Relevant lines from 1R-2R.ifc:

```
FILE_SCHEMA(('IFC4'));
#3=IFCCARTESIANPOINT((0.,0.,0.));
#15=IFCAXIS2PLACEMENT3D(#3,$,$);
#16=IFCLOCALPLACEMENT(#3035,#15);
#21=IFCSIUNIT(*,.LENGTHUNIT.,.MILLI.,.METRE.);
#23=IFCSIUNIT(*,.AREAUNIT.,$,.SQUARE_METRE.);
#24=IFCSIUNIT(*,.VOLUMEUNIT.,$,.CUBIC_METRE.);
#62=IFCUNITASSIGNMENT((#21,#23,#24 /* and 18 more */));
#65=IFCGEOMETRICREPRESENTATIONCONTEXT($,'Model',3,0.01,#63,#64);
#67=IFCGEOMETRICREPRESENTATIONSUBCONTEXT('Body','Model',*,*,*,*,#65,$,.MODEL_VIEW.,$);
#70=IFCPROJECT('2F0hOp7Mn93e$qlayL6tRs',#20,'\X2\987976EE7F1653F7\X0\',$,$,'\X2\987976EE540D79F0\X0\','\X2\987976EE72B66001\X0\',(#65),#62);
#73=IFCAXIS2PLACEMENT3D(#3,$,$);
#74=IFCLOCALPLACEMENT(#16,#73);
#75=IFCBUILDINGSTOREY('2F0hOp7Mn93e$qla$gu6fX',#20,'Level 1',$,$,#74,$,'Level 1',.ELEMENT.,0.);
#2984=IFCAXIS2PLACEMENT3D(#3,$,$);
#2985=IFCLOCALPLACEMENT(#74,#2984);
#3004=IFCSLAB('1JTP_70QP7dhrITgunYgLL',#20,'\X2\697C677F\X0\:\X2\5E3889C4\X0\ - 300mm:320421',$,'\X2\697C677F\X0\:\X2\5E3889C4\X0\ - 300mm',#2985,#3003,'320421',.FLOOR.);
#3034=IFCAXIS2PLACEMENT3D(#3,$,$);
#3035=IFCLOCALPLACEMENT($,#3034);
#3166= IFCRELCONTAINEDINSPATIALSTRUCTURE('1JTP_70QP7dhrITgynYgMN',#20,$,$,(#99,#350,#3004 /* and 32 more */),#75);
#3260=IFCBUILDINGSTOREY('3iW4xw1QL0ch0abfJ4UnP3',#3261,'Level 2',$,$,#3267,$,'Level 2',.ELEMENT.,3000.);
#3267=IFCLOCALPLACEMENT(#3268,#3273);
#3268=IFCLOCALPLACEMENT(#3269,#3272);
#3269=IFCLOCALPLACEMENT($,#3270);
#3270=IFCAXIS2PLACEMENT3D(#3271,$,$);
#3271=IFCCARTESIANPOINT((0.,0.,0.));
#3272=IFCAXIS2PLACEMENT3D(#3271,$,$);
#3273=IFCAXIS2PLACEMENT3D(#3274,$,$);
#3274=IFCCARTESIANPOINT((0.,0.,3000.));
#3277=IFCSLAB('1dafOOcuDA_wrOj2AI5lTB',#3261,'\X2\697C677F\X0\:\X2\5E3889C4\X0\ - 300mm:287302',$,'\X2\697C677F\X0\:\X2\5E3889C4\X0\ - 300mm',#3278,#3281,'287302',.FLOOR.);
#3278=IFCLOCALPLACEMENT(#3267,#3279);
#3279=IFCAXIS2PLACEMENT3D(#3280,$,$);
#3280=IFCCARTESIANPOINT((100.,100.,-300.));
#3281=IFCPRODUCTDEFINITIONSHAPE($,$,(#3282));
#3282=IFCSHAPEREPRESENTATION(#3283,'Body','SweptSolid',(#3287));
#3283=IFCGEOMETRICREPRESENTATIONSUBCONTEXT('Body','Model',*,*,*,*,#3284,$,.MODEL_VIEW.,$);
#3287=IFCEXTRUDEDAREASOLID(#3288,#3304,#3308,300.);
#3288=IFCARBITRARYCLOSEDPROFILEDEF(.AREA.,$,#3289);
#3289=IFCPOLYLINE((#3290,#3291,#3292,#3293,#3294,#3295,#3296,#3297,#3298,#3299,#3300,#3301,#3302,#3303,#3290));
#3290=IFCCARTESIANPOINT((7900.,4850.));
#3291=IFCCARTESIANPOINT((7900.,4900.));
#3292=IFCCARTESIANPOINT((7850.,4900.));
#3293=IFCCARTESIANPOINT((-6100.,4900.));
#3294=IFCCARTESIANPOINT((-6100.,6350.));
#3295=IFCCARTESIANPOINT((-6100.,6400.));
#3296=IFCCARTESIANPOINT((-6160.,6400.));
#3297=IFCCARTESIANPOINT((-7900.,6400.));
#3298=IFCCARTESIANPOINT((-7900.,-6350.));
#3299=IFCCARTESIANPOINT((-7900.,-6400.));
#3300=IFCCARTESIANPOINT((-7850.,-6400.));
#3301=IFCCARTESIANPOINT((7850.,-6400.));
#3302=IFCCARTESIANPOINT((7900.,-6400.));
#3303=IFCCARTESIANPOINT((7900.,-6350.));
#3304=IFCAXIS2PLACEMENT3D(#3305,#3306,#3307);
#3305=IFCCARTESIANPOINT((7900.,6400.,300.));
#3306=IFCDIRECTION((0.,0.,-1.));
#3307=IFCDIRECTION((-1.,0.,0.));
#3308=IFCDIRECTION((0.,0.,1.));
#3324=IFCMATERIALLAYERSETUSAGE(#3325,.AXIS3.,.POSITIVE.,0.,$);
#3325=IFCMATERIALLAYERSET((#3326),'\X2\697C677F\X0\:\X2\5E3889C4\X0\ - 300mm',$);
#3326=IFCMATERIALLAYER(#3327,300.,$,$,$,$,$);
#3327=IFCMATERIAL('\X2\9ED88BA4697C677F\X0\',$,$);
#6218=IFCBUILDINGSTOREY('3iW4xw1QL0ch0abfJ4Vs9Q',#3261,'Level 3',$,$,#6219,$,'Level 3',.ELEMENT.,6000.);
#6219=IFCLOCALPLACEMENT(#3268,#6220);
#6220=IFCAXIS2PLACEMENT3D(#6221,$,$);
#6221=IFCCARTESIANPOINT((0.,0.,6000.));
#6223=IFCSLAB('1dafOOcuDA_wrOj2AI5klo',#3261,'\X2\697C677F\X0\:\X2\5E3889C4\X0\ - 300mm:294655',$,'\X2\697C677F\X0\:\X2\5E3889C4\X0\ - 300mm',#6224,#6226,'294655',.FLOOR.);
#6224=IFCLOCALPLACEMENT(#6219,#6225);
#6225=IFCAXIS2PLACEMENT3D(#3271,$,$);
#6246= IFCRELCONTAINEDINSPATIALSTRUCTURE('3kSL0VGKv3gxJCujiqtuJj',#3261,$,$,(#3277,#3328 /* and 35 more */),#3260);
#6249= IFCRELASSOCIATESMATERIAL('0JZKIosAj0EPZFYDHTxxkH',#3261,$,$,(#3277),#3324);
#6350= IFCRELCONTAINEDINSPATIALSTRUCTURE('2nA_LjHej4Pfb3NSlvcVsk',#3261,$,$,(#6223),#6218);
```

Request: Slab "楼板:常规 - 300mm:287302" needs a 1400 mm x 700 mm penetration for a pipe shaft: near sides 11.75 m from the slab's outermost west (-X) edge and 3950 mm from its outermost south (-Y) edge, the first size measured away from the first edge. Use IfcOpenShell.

```python
import numpy as np
import ifcopenshell
import ifcopenshell.api.feature
import ifcopenshell.api.geometry
import ifcopenshell.api.root
import ifcopenshell.geom
import ifcopenshell.util.placement
import ifcopenshell.util.representation
import ifcopenshell.util.shape
import ifcopenshell.util.unit

model = ifcopenshell.open("1R-2R.ifc")
unit_scale = ifcopenshell.util.unit.calculate_unit_scale(model)
settings = ifcopenshell.geom.settings()


def volume(element):
    """Net volume in cubic metres, openings subtracted."""
    shape = ifcopenshell.geom.create_shape(settings, element)
    return ifcopenshell.util.shape.get_volume(shape.geometry)


slab = model.by_guid("1dafOOcuDA_wrOj2AI5lTB")
before = volume(slab)

# Extent in the slab's own axes, in metres. The edges named are its -X and -Y sides.
slab_shape = ifcopenshell.geom.create_shape(settings, slab)
vertices = ifcopenshell.util.shape.get_vertices(slab_shape.geometry)
x_min, y_min, bottom = vertices.min(axis=0)
top = vertices[:, 2].max()

opening = ifcopenshell.api.root.create_entity(model, ifc_class="IfcOpeningElement", name="Pipe shaft opening", predefined_type="OPENING")
context = ifcopenshell.util.representation.get_context(model, "Model", "Body", "MODEL_VIEW")
width, depth = 1.4, 0.7
outline = [(0.0, 0.0), (width, 0.0), (width, depth), (0.0, depth), (0.0, 0.0)]
# Overshoot both faces by 50 mm so the cut is clean.
shape = ifcopenshell.api.geometry.add_slab_representation(
    model, context=context, depth=top - bottom + 0.1, polyline=outline
)
ifcopenshell.api.geometry.assign_representation(model, product=opening, representation=shape)

matrix = ifcopenshell.util.placement.get_local_placement(slab.ObjectPlacement)
matrix[:, 3] = matrix @ np.append(np.array([x_min + 11.75, y_min + 3.95, bottom - 0.05]) / unit_scale, 1.0)
ifcopenshell.api.geometry.edit_object_placement(model, product=opening, matrix=matrix, is_si=False)
ifcopenshell.api.feature.add_feature(model, feature=opening, element=slab)

after = volume(slab)

print(f"slab volume {before:.3f} -> {after:.3f} m3")

model.write("1R-2R-out.ifc")
```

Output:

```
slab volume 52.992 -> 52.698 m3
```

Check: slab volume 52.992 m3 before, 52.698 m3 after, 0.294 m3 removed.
